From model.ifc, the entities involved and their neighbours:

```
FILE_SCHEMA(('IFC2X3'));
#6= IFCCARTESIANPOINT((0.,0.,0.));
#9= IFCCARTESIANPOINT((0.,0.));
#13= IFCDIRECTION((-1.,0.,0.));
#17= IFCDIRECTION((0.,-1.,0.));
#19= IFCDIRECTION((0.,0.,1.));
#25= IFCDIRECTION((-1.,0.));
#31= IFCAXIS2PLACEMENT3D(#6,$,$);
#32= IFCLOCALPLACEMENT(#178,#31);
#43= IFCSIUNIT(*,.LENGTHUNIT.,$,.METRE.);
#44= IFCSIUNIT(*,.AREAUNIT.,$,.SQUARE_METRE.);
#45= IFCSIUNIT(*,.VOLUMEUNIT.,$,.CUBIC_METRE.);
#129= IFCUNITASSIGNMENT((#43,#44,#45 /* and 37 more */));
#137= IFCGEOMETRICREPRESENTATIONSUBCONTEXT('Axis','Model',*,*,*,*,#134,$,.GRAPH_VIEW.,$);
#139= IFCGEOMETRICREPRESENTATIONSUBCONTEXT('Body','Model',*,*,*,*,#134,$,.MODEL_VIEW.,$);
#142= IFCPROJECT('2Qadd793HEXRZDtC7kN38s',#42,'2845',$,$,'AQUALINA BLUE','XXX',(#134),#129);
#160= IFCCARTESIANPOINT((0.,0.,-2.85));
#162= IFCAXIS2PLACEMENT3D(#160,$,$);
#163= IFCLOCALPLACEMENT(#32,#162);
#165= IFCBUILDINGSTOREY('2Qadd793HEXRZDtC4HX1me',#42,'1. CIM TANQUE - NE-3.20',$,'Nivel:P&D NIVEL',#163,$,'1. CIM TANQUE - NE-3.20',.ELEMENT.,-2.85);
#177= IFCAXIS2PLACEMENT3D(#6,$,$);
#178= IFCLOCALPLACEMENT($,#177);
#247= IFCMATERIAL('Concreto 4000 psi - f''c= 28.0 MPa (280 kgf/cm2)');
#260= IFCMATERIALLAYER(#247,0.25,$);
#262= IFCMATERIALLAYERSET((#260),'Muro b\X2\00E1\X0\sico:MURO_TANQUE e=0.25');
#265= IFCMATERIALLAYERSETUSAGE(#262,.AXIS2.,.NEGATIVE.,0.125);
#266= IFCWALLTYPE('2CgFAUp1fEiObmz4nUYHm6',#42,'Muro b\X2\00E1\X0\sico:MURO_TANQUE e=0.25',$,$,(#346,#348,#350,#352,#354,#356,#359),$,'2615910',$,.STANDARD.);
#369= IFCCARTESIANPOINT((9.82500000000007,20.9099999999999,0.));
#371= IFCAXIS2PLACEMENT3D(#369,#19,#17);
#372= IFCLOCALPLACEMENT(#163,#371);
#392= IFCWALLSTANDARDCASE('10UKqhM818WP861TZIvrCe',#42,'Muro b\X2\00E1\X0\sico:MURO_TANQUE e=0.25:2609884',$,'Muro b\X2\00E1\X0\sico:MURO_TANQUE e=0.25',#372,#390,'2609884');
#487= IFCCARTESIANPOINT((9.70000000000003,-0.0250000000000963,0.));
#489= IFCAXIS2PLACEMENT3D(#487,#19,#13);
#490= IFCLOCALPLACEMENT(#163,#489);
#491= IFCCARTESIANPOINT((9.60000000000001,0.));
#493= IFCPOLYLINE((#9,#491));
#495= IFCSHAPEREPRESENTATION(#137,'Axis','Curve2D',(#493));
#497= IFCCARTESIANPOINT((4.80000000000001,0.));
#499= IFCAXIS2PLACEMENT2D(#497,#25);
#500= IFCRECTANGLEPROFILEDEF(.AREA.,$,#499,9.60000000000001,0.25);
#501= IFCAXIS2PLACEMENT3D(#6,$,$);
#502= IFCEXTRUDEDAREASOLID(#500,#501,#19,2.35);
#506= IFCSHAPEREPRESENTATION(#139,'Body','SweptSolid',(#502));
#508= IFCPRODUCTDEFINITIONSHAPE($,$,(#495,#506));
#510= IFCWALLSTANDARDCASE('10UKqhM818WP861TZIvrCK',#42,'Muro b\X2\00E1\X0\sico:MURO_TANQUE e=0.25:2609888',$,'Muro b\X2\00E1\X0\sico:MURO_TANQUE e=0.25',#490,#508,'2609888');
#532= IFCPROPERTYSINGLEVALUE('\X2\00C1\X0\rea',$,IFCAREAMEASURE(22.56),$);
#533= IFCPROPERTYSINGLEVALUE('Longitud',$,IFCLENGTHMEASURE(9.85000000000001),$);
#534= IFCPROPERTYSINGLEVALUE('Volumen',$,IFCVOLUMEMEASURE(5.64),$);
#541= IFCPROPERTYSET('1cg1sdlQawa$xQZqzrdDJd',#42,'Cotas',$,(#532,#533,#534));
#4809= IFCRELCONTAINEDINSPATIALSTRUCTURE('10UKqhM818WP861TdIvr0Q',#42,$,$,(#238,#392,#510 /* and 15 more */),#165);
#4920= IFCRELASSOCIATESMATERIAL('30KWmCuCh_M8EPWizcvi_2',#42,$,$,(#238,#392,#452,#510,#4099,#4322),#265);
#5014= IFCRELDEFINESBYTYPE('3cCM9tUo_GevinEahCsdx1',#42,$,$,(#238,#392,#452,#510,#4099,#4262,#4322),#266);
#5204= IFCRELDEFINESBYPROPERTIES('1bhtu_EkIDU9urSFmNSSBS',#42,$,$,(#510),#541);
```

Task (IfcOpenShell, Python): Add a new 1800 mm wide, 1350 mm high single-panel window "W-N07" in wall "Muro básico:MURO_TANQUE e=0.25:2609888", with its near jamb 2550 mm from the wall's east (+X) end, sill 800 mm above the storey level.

```python
import numpy as np
import ifcopenshell
import ifcopenshell.api.feature
import ifcopenshell.api.geometry
import ifcopenshell.api.pset
import ifcopenshell.api.root
import ifcopenshell.api.spatial
import ifcopenshell.api.type
import ifcopenshell.geom
import ifcopenshell.util.element
import ifcopenshell.util.placement
import ifcopenshell.util.representation
import ifcopenshell.util.shape
import ifcopenshell.util.unit

model = ifcopenshell.open("model.ifc")
unit_scale = ifcopenshell.util.unit.calculate_unit_scale(model)
area_scale = ifcopenshell.util.unit.calculate_unit_scale(model, "AREAUNIT")
volume_scale = ifcopenshell.util.unit.calculate_unit_scale(model, "VOLUMEUNIT")
settings = ifcopenshell.geom.settings()


def volume(element):
    """Net volume in cubic metres, openings subtracted."""
    shape = ifcopenshell.geom.create_shape(settings, element)
    return ifcopenshell.util.shape.get_volume(shape.geometry)


wall = model.by_guid("10UKqhM818WP861TZIvrCK")
storey = ifcopenshell.util.element.get_container(wall, ifc_class="IfcBuildingStorey")
context = ifcopenshell.util.representation.get_context(model, "Model", "Body", "MODEL_VIEW")
before = volume(wall)

width, height, from_end, sill = 1.8, 1.35, 2.55, 0.8  # metres

# The wall runs along its own X axis, and the end named is its -X end.
wall_shape = ifcopenshell.geom.create_shape(settings, wall)
x, y, z = ifcopenshell.util.shape.get_vertices(wall_shape.geometry).T
start = x.min() + from_end
face, thickness = float(y.min()), float(y.max() - y.min())
wall_matrix = ifcopenshell.util.placement.get_local_placement(wall.ObjectPlacement)
level = ifcopenshell.util.placement.get_local_placement(storey.ObjectPlacement)[2, 3]


def in_wall(x, y):
    """Placement at x, y metres in the wall's axes, at sill height."""
    matrix = wall_matrix.copy()
    matrix[:, 3] = wall_matrix @ np.array([x / unit_scale, y / unit_scale, 0.0, 1.0])
    matrix[2, 3] = level + sill / unit_scale
    return matrix


# Opening: a box that overshoots both wall faces by 50 mm.
opening = ifcopenshell.api.root.create_entity(model, ifc_class="IfcOpeningElement")
box = ifcopenshell.api.geometry.add_wall_representation(
    model, context=context, length=width, height=height, thickness=thickness + 0.1
)
ifcopenshell.api.geometry.assign_representation(model, product=opening, representation=box)
ifcopenshell.api.geometry.edit_object_placement(model, product=opening, matrix=in_wall(start, face - 0.05), is_si=False)
ifcopenshell.api.feature.add_feature(model, feature=opening, element=wall)

window = ifcopenshell.api.root.create_entity(model, ifc_class="IfcWindow", name="W-N07")
window.OverallWidth, window.OverallHeight = width / unit_scale, height / unit_scale
body = ifcopenshell.api.geometry.add_window_representation(
    model,
    context=context,
    overall_width=window.OverallWidth,
    overall_height=window.OverallHeight,
    partition_type="SINGLE_PANEL",
)
ifcopenshell.api.geometry.assign_representation(model, product=window, representation=body)
ifcopenshell.api.spatial.assign_container(model, products=[window], relating_structure=storey)
fills = ifcopenshell.api.feature.add_filling(model, opening=opening, element=window)
fills.OwnerHistory = window.OwnerHistory  # required in IFC2X3

# IFC2X3 keeps the operation on the window style.
style = ifcopenshell.api.root.create_entity(model, ifc_class="IfcWindowStyle", name="W-N07")
style.OperationType, style.ConstructionType = "SINGLE_PANEL", "NOTDEFINED"
style.ParameterTakesPrecedence = style.Sizeable = False
ifcopenshell.api.type.assign_type(model, related_objects=[window], relating_type=style)

# Centre the window in the wall's thickness.
ifcopenshell.api.geometry.edit_object_placement(model, product=window, matrix=in_wall(start, face), is_si=False)
window_shape = ifcopenshell.geom.create_shape(settings, window)
depth = ifcopenshell.util.shape.get_vertices(window_shape.geometry)[:, 1]
offset = face + thickness / 2 - (depth.min() + depth.max()) / 2
ifcopenshell.api.geometry.edit_object_placement(model, product=window, matrix=in_wall(start, offset), is_si=False)

after = volume(wall)

# Update the wall's stored quantities.
pset = model.by_id(ifcopenshell.util.element.get_pset(wall, "Cotas", should_inherit=False)["id"])
ifcopenshell.api.pset.edit_pset(model, pset=pset, properties={
    "Área": model.create_entity("IfcAreaMeasure", after / thickness / area_scale),
    "Volumen": model.create_entity("IfcVolumeMeasure", after / volume_scale),
})

print(f"wall volume {before:.3f} -> {after:.3f} m3")

model.write("model-out.ifc")
```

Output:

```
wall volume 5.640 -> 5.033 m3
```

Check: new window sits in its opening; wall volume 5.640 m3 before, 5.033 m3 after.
